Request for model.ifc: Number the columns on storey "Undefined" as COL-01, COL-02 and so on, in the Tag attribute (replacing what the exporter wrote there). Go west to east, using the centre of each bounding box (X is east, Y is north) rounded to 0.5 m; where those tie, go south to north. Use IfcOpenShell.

First a look at what the model holds.

```python
import ifcopenshell
import ifcopenshell.util.element
import ifcopenshell.util.placement

model = ifcopenshell.open("model.ifc")
print(model.schema)
storey = next(s for s in model.by_type("IfcBuildingStorey") if s.Name == "Undefined")
columns = [e for e in ifcopenshell.util.element.get_decomposition(storey) if e.is_a("IfcColumn")]
for e in sorted(columns, key=lambda e: e.id()):
    origin = ifcopenshell.util.placement.get_local_placement(e.ObjectPlacement)[:3, 3]
    print(e.id(), e.Tag, e.Name, origin.round(2) + 0.0, sep=" | ")
```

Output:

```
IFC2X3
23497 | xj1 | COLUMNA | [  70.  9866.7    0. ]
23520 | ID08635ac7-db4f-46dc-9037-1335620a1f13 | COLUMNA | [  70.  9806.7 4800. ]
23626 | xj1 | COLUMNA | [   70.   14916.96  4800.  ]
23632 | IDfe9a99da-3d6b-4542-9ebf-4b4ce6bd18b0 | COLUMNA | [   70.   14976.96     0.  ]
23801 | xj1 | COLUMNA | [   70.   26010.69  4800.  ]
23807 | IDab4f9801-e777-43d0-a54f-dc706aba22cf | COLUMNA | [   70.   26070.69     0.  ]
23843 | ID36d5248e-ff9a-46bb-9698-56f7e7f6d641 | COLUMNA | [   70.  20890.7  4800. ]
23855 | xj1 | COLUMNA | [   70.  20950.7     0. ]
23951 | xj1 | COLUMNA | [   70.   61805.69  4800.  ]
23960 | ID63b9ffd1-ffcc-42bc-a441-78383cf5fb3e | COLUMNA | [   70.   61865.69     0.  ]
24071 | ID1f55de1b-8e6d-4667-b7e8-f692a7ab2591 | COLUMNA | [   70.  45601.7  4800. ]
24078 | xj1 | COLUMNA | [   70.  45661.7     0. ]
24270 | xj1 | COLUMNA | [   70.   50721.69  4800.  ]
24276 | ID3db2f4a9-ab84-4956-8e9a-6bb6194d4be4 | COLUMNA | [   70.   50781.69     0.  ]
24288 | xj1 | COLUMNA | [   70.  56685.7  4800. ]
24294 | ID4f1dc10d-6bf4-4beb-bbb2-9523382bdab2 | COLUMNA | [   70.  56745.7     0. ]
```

```python
import ifcopenshell
import ifcopenshell.geom
import ifcopenshell.util.element
import ifcopenshell.util.shape

model = ifcopenshell.open("model.ifc")
settings = ifcopenshell.geom.settings()
settings.set("use-world-coords", True)


def centre(element):
    shape = ifcopenshell.geom.create_shape(settings, element)
    return ifcopenshell.util.shape.get_bbox_centroid(shape.geometry)


storey = next(s for s in model.by_type("IfcBuildingStorey") if s.Name == "Undefined")
columns = [e for e in ifcopenshell.util.element.get_decomposition(storey) if e.is_a("IfcColumn")]

# Insertion points can sit at a corner or the storey origin, so sort by the geometry (in metres).
centres = {e: centre(e) for e in columns}
columns.sort(key=lambda e: (round(centres[e][0] / 0.5), centres[e][1]))

for i, e in enumerate(columns, start=1):
    number = f"COL-{i:02d}"
    e.Tag = number
    print(e.id(), number)

model.write("model_updated.ifc")
```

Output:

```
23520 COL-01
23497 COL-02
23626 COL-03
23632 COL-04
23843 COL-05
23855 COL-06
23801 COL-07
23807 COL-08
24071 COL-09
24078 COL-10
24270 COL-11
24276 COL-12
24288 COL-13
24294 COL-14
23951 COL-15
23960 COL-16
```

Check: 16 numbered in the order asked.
